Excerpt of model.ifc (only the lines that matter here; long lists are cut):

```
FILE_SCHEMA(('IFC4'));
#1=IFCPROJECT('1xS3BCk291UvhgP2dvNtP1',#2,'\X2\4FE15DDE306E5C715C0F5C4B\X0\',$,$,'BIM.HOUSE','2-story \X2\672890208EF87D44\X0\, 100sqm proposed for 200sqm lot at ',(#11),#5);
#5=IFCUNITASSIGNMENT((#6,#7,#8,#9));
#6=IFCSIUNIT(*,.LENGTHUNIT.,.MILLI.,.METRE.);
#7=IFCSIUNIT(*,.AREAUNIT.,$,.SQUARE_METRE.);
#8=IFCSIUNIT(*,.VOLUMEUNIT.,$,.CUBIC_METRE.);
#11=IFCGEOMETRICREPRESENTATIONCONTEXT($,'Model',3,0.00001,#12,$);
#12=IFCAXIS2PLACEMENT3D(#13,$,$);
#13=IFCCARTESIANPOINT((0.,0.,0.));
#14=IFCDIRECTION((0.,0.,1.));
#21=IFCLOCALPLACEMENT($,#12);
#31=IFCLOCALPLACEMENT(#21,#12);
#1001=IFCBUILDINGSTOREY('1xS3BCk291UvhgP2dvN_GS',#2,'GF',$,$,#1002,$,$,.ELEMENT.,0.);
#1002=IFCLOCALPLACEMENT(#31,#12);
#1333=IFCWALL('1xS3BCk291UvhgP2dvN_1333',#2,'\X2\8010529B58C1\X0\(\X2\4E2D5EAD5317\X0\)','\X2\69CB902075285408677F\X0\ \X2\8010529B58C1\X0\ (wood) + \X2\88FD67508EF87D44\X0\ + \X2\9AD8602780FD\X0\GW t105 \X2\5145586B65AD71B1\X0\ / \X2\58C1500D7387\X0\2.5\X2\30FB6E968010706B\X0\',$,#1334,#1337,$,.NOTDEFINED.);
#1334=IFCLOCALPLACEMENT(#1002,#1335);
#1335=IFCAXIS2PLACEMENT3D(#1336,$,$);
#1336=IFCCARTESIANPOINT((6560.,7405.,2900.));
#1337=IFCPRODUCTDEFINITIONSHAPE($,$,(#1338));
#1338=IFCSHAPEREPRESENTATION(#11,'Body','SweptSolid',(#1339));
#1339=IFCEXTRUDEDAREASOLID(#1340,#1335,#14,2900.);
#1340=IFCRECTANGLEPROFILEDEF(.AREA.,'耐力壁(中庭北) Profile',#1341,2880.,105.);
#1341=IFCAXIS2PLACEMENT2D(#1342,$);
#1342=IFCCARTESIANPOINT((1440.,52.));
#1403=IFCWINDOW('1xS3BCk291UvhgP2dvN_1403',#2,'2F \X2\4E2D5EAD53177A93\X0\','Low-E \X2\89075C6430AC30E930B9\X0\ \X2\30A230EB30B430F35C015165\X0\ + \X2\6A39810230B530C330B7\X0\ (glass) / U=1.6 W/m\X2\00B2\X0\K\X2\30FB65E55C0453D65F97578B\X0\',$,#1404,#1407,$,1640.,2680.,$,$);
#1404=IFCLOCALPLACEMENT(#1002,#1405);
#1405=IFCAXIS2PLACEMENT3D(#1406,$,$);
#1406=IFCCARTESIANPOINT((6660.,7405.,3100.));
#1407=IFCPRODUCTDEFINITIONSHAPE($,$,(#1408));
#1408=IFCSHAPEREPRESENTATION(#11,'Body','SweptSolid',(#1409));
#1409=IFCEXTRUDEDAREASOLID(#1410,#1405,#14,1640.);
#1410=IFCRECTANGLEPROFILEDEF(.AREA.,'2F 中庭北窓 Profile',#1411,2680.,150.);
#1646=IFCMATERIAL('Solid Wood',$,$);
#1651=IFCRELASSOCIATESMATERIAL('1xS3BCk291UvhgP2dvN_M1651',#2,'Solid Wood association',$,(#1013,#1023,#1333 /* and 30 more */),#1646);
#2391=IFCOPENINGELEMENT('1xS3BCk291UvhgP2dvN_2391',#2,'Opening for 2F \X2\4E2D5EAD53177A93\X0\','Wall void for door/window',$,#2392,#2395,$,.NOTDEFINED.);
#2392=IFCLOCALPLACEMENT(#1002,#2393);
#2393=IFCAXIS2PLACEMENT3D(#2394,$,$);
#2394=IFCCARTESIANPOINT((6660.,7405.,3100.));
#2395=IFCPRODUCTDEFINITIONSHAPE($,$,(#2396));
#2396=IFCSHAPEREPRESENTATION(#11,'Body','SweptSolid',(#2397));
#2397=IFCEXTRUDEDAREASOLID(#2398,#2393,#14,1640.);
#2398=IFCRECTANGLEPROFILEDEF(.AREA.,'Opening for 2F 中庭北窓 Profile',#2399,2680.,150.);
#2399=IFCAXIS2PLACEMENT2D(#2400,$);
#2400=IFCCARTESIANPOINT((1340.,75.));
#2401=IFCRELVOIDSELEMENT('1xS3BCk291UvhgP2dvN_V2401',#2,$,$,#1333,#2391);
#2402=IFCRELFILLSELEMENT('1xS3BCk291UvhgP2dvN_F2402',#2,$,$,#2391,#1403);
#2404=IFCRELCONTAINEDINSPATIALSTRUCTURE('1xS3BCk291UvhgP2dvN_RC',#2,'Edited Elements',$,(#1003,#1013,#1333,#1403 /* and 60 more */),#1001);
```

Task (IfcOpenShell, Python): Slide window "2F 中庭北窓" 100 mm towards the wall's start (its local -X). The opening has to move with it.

```python
import ifcopenshell
import ifcopenshell.api.geometry
import ifcopenshell.util.placement

model = ifcopenshell.open("model.ifc")

window = model.by_id(1403)
opening = window.FillsVoids[0].RelatingOpeningElement
wall = opening.VoidsElements[0].RelatingBuildingElement

wall_matrix = ifcopenshell.util.placement.get_local_placement(wall.ObjectPlacement)
shift = wall_matrix[:3, 0] * -100.0
before = ifcopenshell.util.placement.get_local_placement(window.ObjectPlacement)[:3, 3].copy()

# The window is not placed relative to its opening, so move both.
for product in (opening, window):
    matrix = ifcopenshell.util.placement.get_local_placement(product.ObjectPlacement)
    matrix[:3, 3] += shift
    ifcopenshell.api.geometry.edit_object_placement(model, product=product, matrix=matrix, is_si=False)

after = ifcopenshell.util.placement.get_local_placement(window.ObjectPlacement)[:3, 3]
print("window moved by", (after - before).round(3) + 0.0)

model.write("model_v2.ifc")
```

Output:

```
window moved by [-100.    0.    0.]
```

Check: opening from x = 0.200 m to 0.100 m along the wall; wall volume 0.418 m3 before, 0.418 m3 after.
